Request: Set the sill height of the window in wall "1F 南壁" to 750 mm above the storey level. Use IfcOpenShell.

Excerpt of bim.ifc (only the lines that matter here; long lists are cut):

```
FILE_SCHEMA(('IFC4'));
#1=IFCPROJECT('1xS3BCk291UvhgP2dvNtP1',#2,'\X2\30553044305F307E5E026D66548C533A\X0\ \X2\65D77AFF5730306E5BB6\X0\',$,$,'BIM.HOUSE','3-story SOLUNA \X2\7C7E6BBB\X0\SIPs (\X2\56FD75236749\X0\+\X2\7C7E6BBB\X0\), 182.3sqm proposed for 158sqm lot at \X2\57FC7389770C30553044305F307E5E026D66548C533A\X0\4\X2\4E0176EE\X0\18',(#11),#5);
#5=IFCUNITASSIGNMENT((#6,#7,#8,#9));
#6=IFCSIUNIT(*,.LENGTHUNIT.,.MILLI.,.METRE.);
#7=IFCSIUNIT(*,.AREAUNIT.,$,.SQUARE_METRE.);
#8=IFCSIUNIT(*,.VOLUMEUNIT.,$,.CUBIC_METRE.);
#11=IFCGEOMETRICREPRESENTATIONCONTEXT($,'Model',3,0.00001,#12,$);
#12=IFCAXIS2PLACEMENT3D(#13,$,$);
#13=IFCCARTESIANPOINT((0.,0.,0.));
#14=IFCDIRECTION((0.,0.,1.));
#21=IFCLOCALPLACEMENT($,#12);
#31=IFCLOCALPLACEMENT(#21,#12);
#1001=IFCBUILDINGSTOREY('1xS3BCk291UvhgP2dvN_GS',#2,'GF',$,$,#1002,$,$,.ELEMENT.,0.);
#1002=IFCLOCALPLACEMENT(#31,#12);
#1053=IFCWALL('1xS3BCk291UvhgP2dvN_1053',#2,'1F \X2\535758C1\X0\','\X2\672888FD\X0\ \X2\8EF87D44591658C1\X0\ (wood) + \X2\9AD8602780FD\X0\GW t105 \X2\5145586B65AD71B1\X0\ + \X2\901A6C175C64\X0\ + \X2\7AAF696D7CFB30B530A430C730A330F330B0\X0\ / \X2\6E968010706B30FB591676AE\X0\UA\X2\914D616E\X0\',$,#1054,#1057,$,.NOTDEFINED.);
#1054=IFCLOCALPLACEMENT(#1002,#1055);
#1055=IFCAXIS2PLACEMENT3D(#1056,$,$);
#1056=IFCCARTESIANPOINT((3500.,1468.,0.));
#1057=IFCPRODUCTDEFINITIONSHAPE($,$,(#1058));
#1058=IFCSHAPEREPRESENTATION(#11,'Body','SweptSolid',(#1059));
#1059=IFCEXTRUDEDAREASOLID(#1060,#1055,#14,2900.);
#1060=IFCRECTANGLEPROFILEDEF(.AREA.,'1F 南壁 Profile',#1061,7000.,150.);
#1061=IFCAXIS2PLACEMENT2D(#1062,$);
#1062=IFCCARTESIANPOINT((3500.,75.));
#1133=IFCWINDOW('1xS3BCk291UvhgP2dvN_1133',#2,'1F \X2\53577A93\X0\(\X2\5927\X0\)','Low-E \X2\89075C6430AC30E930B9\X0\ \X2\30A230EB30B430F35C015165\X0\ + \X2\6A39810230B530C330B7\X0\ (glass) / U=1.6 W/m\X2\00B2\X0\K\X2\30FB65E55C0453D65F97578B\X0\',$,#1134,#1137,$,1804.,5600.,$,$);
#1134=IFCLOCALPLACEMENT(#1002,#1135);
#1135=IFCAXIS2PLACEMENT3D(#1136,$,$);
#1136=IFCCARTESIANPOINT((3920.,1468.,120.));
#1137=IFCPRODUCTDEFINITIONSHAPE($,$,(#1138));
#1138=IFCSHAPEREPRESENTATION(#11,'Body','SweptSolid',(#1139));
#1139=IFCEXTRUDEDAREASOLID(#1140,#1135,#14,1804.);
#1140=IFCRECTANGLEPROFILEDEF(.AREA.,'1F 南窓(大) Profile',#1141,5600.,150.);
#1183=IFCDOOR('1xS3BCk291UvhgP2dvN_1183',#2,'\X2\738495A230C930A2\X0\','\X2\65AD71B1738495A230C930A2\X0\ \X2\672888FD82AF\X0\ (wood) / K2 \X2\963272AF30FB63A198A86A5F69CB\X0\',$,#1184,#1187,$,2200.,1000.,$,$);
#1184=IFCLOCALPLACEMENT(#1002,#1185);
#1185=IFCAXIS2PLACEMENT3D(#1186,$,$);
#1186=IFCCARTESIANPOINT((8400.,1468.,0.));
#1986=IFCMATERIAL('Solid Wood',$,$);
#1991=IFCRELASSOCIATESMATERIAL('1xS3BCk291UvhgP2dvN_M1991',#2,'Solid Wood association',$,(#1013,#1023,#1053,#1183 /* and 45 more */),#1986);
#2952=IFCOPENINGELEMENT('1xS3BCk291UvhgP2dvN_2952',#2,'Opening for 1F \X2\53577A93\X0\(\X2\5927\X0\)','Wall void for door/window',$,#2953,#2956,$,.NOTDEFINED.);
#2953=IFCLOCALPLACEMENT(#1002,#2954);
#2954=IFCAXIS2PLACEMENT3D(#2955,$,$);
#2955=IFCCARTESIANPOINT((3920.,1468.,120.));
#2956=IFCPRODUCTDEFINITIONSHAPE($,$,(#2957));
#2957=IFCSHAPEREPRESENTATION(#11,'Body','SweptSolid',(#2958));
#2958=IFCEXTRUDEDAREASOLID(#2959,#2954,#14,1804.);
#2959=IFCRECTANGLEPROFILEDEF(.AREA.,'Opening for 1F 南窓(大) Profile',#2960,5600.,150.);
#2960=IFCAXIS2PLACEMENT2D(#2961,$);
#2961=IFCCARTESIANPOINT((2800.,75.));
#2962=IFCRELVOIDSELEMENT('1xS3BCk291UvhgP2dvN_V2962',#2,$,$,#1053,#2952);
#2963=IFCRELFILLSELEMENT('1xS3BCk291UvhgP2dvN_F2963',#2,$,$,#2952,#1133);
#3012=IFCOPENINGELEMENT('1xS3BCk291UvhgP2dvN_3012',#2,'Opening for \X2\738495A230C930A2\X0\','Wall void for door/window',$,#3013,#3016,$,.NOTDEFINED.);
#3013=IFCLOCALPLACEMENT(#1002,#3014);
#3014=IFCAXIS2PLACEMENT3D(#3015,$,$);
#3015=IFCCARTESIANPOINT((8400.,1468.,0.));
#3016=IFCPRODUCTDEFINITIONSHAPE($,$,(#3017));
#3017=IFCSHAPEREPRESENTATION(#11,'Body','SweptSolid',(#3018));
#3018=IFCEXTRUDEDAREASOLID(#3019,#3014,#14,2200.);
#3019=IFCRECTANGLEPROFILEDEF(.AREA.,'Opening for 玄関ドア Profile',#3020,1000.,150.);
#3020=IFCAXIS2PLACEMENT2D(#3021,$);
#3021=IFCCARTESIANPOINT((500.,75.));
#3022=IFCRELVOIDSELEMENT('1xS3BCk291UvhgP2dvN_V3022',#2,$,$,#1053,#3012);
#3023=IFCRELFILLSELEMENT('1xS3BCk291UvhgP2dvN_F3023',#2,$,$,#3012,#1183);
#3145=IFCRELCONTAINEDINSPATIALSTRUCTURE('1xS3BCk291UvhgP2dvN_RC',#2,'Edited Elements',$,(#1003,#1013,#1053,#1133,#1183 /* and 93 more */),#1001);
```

```python
import numpy as np
import ifcopenshell
import ifcopenshell.api.geometry
import ifcopenshell.geom
import ifcopenshell.util.element
import ifcopenshell.util.placement
import ifcopenshell.util.shape
import ifcopenshell.util.unit

model = ifcopenshell.open("bim.ifc")
unit_scale = ifcopenshell.util.unit.calculate_unit_scale(model)

window = model.by_guid("1xS3BCk291UvhgP2dvN_1133")
opening = window.FillsVoids[0].RelatingOpeningElement
storey = ifcopenshell.util.element.get_container(window, ifc_class="IfcBuildingStorey")
level = ifcopenshell.util.placement.get_local_placement(storey.ObjectPlacement)[2, 3]

# The opening's origin need not be at the sill, so measure its lowest point.
shape = ifcopenshell.geom.create_shape(ifcopenshell.geom.settings(), opening)
bottom = ifcopenshell.util.shape.get_shape_bottom_elevation(shape, shape.geometry) / unit_scale
dz = level + 750.0 - bottom

shift = np.array([0.0, 0.0, dz])
# The window is not placed relative to its opening, so move both.
for product in (opening, window):
    matrix = ifcopenshell.util.placement.get_local_placement(product.ObjectPlacement)
    matrix[:3, 3] += shift
    ifcopenshell.api.geometry.edit_object_placement(model, product=product, matrix=matrix, is_si=False)

print(f"moved by {dz * unit_scale:+.3f} m")

model.write("bim-out.ifc")
```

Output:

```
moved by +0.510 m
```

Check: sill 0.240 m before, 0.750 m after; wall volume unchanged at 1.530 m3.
